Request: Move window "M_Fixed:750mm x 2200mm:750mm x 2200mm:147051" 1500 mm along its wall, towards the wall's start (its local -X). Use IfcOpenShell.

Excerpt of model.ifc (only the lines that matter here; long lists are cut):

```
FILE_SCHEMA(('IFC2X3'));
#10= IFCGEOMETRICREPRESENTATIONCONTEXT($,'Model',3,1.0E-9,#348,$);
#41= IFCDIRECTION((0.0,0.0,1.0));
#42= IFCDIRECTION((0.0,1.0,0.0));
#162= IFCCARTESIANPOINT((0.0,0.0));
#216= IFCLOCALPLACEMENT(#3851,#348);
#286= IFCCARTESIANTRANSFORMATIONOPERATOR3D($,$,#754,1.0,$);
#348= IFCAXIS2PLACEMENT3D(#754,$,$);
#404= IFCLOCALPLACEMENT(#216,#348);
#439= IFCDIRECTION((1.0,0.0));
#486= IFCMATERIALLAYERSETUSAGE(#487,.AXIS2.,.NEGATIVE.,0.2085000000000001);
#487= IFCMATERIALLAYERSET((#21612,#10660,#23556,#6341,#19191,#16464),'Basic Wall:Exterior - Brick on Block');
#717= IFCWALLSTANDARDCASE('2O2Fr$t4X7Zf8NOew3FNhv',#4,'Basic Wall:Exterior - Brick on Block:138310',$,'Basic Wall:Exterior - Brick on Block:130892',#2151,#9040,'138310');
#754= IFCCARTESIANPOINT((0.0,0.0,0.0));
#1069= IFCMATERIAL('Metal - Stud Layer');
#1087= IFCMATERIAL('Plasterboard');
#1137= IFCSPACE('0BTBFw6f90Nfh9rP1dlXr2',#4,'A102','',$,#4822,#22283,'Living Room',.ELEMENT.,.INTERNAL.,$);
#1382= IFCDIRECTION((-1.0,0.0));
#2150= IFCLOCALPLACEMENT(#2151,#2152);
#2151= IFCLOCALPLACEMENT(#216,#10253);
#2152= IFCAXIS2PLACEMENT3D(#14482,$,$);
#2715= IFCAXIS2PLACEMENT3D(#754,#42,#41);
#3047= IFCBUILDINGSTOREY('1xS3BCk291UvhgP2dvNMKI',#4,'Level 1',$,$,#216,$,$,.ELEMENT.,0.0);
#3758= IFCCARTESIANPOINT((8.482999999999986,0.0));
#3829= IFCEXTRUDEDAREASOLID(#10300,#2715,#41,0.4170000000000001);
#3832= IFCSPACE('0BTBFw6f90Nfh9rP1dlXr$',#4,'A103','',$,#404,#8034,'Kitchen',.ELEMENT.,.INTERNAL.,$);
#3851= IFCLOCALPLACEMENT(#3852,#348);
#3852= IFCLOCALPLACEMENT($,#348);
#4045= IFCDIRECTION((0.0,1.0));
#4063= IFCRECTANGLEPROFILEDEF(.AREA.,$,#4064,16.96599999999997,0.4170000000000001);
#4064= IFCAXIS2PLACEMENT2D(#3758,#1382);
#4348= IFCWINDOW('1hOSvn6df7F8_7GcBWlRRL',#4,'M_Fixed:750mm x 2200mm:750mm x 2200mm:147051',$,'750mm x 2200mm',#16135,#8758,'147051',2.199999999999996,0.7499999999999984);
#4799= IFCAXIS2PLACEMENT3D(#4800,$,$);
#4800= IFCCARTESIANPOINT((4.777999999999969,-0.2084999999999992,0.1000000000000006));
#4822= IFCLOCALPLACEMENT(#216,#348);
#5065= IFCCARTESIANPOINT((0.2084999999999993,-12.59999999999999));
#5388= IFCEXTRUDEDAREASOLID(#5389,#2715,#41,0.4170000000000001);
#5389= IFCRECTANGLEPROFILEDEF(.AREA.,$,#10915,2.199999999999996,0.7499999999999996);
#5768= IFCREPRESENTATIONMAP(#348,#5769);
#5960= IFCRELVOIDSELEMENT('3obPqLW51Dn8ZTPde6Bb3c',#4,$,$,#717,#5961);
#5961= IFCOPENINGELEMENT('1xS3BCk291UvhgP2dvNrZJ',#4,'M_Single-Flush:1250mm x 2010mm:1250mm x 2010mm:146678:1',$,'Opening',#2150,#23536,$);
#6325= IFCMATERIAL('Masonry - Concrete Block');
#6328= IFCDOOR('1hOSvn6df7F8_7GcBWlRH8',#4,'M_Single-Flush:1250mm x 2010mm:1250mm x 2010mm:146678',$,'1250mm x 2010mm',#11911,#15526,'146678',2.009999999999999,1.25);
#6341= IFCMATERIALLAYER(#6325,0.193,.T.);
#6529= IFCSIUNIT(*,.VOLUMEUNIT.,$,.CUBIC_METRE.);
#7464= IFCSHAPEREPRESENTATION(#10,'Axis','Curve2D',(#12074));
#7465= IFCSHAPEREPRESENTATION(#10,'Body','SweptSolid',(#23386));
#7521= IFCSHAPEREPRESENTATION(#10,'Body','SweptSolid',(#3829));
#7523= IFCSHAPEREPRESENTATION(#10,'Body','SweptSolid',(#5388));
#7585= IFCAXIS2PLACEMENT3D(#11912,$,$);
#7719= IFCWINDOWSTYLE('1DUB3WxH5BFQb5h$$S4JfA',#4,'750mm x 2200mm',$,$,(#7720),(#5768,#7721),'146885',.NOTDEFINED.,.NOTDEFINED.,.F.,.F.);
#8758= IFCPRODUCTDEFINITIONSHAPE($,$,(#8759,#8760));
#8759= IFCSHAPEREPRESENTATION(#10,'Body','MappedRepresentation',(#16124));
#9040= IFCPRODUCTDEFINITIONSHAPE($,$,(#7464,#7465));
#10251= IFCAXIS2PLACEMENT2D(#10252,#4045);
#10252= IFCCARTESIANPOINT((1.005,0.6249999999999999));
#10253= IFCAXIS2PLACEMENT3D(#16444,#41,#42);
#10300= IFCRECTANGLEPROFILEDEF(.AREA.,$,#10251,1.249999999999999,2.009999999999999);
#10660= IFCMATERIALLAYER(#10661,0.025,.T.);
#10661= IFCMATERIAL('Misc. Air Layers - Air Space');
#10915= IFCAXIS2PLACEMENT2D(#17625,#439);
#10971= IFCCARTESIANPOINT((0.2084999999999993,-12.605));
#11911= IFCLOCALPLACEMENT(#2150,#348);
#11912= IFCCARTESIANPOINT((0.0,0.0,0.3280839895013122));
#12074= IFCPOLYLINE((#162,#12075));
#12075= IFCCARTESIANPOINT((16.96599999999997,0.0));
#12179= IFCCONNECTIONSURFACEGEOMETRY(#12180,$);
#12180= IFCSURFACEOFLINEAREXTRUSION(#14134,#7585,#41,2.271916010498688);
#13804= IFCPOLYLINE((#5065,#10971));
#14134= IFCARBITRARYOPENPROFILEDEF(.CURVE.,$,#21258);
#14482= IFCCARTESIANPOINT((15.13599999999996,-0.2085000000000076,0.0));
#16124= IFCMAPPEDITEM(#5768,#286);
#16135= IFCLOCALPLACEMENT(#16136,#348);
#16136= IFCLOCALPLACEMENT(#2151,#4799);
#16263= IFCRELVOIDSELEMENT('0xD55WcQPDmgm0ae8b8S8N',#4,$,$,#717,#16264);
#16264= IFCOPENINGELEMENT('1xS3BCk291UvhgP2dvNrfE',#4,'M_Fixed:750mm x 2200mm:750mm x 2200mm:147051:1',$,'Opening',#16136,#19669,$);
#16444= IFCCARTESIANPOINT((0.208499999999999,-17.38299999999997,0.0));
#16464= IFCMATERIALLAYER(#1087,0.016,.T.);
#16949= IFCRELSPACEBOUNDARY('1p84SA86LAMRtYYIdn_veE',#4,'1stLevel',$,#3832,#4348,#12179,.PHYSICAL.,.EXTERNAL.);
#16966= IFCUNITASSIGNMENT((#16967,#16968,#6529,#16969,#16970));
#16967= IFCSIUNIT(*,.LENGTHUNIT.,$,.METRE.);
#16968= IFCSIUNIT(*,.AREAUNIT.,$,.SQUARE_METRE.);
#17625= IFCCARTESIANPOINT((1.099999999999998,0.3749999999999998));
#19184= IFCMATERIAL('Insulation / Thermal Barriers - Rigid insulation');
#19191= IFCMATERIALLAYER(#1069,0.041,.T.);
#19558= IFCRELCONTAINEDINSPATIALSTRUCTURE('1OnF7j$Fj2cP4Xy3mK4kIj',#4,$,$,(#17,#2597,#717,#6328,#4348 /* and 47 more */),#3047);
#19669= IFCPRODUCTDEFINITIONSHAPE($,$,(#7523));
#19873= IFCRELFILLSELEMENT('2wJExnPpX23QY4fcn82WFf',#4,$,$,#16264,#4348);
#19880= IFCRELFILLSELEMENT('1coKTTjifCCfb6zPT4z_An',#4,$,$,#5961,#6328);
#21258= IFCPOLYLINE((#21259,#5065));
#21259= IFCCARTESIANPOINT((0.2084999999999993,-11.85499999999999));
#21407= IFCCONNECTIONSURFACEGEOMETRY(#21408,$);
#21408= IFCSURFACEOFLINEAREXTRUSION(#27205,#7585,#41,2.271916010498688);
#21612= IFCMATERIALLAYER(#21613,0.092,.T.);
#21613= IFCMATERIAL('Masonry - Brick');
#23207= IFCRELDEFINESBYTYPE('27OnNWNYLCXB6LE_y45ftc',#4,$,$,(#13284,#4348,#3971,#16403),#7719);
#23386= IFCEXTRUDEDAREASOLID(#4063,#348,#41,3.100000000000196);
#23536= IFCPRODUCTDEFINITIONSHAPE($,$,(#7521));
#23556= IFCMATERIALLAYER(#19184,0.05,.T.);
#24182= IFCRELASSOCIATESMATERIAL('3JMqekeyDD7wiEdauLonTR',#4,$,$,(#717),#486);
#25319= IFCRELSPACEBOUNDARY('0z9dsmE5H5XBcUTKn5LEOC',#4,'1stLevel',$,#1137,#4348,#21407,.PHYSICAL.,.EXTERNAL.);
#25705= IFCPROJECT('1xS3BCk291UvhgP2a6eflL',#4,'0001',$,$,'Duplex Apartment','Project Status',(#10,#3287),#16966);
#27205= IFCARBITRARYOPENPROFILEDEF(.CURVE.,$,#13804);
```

```python
import numpy as np
import ifcopenshell
import ifcopenshell.api.geometry
import ifcopenshell.util.placement

model = ifcopenshell.open("model.ifc")

window = model.by_id(4348)
opening = window.FillsVoids[0].RelatingOpeningElement
wall = opening.VoidsElements[0].RelatingBuildingElement

wall_matrix = ifcopenshell.util.placement.get_local_placement(wall.ObjectPlacement)
shift = wall_matrix[:3, 0] * -1.5
before = ifcopenshell.util.placement.get_local_placement(window.ObjectPlacement)[:3, 3].copy()

# The window is placed relative to its opening, so it follows when the opening moves.
matrix = ifcopenshell.util.placement.get_local_placement(opening.ObjectPlacement)
matrix[:3, 3] += shift
ifcopenshell.api.geometry.edit_object_placement(
    model, product=opening, matrix=matrix, is_si=False, should_transform_children=True
)

# Space boundary surfaces are stored in each space's coordinates; move them too.
for rel in window.ProvidesBoundaries:
    if not rel.ConnectionGeometry:
        continue
    surface = rel.ConnectionGeometry.SurfaceOnRelatingElement
    space_matrix = ifcopenshell.util.placement.get_local_placement(rel.RelatingSpace.ObjectPlacement)
    point = np.array(surface.Position.Location.Coordinates) + space_matrix[:3, :3].T @ shift
    surface.Position = model.createIfcAxis2Placement3D(
        model.createIfcCartesianPoint(point.tolist()), surface.Position.Axis, surface.Position.RefDirection
    )

after = ifcopenshell.util.placement.get_local_placement(window.ObjectPlacement)[:3, 3]
print("window moved by", (after - before).round(3) + 0.0)

model.write("model_updated.ifc")
```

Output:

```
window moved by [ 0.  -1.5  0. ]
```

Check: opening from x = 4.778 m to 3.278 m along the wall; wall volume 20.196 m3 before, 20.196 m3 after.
